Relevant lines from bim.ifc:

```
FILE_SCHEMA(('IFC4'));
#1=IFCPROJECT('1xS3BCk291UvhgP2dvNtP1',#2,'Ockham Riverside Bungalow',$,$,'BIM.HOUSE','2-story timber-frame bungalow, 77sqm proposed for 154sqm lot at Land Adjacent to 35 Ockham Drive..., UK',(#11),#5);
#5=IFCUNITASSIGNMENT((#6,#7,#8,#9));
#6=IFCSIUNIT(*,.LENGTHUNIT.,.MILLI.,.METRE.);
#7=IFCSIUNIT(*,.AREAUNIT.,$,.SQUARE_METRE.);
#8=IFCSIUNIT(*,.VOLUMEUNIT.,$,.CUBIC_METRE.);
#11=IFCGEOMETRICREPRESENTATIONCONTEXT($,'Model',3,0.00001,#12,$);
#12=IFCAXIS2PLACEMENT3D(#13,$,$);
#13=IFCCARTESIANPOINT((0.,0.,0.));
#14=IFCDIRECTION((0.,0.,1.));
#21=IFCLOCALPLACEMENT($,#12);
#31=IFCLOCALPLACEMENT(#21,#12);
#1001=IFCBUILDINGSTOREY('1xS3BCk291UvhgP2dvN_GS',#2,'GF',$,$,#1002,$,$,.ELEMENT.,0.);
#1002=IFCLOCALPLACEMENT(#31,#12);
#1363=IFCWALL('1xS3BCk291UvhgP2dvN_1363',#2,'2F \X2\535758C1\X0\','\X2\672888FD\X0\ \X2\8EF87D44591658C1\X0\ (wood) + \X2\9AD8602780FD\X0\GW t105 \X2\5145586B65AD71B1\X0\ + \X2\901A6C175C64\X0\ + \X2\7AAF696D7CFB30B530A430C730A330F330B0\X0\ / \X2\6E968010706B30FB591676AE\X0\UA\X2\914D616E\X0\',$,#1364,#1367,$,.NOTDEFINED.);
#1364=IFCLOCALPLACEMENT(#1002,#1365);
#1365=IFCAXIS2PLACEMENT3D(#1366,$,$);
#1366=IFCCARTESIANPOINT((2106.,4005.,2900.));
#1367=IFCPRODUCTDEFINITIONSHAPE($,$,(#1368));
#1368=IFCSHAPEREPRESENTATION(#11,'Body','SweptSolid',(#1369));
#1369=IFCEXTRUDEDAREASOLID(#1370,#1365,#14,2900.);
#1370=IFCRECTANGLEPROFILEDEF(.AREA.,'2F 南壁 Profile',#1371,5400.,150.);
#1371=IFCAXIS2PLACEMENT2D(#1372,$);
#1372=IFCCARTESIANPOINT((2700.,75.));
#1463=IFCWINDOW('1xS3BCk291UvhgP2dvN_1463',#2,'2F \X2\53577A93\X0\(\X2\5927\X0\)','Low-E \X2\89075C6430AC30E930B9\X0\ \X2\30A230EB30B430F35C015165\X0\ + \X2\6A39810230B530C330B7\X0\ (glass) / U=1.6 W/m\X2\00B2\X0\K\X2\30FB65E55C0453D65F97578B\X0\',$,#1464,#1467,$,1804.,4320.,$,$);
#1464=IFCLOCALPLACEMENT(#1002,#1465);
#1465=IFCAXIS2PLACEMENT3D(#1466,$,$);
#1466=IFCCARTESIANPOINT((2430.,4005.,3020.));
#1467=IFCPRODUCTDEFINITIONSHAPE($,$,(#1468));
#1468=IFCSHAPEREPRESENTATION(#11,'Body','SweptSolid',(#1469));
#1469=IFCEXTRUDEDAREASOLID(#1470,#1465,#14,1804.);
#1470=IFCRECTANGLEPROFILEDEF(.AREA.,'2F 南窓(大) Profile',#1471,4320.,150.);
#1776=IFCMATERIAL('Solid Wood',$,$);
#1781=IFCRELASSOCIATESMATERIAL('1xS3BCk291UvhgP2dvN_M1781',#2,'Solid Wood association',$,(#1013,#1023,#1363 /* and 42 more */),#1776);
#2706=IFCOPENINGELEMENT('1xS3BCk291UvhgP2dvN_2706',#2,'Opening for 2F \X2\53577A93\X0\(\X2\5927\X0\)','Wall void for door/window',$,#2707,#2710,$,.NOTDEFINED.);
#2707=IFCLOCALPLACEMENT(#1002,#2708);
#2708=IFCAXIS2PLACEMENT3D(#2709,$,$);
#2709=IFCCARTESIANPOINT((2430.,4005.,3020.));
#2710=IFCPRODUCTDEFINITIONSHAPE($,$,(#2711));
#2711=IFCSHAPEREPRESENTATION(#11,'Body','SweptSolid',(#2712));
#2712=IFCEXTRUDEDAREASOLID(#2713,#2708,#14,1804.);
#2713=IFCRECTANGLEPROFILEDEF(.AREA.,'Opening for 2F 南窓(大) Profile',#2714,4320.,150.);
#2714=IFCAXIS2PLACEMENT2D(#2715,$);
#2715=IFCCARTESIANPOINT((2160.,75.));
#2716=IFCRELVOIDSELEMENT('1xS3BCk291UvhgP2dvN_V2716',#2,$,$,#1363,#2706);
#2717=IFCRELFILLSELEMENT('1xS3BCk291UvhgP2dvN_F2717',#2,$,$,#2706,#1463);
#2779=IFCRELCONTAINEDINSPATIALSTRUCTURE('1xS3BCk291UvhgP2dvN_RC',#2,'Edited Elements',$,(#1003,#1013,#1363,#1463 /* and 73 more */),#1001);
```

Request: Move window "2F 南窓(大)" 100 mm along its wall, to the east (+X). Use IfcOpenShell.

```python
import ifcopenshell
import ifcopenshell.api.geometry
import ifcopenshell.util.placement
import ifcopenshell.util.unit

model = ifcopenshell.open("bim.ifc")
unit_scale = ifcopenshell.util.unit.calculate_unit_scale(model)

window = model.by_guid("1xS3BCk291UvhgP2dvN_1463")
opening = window.FillsVoids[0].RelatingOpeningElement
wall = opening.VoidsElements[0].RelatingBuildingElement

wall_matrix = ifcopenshell.util.placement.get_local_placement(wall.ObjectPlacement)
shift = wall_matrix[:3, 0] * 0.1 / unit_scale
before = ifcopenshell.util.placement.get_local_placement(window.ObjectPlacement)[:3, 3].copy()

# The window is not placed relative to its opening, so move both.
for product in (opening, window):
    matrix = ifcopenshell.util.placement.get_local_placement(product.ObjectPlacement)
    matrix[:3, 3] += shift
    ifcopenshell.api.geometry.edit_object_placement(model, product=product, matrix=matrix, is_si=False)

after = ifcopenshell.util.placement.get_local_placement(window.ObjectPlacement)[:3, 3]
print("window moved by", (after - before).round(3) + 0.0)

model.write("bim_edited.ifc")
```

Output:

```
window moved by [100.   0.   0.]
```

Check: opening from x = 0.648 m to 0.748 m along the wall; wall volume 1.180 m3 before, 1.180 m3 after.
